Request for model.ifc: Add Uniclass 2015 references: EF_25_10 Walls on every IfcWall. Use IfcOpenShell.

First a look at what the model holds.

```python
import ifcopenshell

model = ifcopenshell.open("model.ifc")
print(model.schema)
print("classifications:", [c.Name for c in model.by_type("IfcClassification")])
for ifc_class in ("IfcDoor", "IfcRoof", "IfcStair", "IfcWall", "IfcWindow"):
    print(ifc_class, len(model.by_type(ifc_class)))
```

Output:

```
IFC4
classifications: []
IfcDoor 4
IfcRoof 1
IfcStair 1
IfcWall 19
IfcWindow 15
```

```python
import ifcopenshell
import ifcopenshell.api.classification

model = ifcopenshell.open("model.ifc")

system = ifcopenshell.api.classification.add_classification(model, classification="Uniclass 2015")

codes = {
    "IfcWall": ("EF_25_10", "Walls"),
}
for ifc_class, (code, name) in codes.items():
    products = model.by_type(ifc_class)
    ifcopenshell.api.classification.add_reference(
        model, products=products, classification=system, identification=code, name=name
    )
    print(code, len(products))

model.write("model_rev.ifc")
```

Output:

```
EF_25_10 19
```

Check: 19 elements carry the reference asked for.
